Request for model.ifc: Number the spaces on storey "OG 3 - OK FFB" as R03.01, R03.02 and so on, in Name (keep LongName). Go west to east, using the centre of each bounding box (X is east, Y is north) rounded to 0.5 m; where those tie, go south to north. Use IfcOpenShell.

First a look at what the model holds.

```python
import ifcopenshell
import ifcopenshell.util.element
import ifcopenshell.util.placement

model = ifcopenshell.open("model.ifc")
print(model.schema)
storey = next(s for s in model.by_type("IfcBuildingStorey") if s.Name == "OG 3 - OK FFB")
spaces = [e for e in ifcopenshell.util.element.get_decomposition(storey) if e.is_a("IfcSpace")]
for e in sorted(spaces, key=lambda e: e.id()):
    origin = ifcopenshell.util.placement.get_local_placement(e.ObjectPlacement)[:3, 3]
    print(e.id(), e.Name, e.LongName, origin.round(2) + 0.0, sep=" | ")
```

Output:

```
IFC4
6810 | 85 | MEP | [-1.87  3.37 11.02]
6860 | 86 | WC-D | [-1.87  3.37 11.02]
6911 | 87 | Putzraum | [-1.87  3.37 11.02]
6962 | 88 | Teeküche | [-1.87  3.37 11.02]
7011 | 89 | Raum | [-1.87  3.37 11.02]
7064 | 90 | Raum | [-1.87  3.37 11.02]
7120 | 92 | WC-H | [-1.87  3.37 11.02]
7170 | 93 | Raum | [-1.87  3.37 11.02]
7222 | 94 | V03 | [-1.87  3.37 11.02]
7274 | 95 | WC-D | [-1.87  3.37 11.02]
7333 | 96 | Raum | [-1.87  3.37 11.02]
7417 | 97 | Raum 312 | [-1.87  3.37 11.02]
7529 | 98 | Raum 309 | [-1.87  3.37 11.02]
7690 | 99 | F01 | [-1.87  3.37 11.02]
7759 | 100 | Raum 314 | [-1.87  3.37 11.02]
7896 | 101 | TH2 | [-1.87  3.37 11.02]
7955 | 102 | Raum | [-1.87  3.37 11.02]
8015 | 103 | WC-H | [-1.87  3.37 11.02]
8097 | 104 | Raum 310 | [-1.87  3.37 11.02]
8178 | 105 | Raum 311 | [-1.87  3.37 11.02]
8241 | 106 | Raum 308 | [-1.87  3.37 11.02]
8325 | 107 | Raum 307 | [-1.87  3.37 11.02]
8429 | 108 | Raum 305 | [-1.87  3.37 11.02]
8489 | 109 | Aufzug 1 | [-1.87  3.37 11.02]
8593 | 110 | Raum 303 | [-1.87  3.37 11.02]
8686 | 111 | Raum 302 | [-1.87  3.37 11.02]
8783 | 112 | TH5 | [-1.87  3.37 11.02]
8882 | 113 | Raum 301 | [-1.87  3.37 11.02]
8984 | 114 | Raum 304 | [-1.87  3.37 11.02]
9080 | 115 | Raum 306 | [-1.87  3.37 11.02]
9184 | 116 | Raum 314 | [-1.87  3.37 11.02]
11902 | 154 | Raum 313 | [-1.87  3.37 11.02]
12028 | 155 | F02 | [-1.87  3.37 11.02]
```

```python
import ifcopenshell
import ifcopenshell.geom
import ifcopenshell.util.element
import ifcopenshell.util.shape

model = ifcopenshell.open("model.ifc")
settings = ifcopenshell.geom.settings()
settings.set("use-world-coords", True)


def centre(element):
    shape = ifcopenshell.geom.create_shape(settings, element)
    return ifcopenshell.util.shape.get_bbox_centroid(shape.geometry)


storey = next(s for s in model.by_type("IfcBuildingStorey") if s.Name == "OG 3 - OK FFB")
spaces = [e for e in ifcopenshell.util.element.get_decomposition(storey) if e.is_a("IfcSpace")]

# Insertion points can sit at a corner or the storey origin, so sort by the geometry (in metres).
centres = {e: centre(e) for e in spaces}
spaces.sort(key=lambda e: (round(centres[e][0] / 0.5), centres[e][1]))

for i, e in enumerate(spaces, start=1):
    number = f"R03.{i:02d}"
    e.Name = number
    print(e.id(), number)

model.write("model_updated.ifc")
```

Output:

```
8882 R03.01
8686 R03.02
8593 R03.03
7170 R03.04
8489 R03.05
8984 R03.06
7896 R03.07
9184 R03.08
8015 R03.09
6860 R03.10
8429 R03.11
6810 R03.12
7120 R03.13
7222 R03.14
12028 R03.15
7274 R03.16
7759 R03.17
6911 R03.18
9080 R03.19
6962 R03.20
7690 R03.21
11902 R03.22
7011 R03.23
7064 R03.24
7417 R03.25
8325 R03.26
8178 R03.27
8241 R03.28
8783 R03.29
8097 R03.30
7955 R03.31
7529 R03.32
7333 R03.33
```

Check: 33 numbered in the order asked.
